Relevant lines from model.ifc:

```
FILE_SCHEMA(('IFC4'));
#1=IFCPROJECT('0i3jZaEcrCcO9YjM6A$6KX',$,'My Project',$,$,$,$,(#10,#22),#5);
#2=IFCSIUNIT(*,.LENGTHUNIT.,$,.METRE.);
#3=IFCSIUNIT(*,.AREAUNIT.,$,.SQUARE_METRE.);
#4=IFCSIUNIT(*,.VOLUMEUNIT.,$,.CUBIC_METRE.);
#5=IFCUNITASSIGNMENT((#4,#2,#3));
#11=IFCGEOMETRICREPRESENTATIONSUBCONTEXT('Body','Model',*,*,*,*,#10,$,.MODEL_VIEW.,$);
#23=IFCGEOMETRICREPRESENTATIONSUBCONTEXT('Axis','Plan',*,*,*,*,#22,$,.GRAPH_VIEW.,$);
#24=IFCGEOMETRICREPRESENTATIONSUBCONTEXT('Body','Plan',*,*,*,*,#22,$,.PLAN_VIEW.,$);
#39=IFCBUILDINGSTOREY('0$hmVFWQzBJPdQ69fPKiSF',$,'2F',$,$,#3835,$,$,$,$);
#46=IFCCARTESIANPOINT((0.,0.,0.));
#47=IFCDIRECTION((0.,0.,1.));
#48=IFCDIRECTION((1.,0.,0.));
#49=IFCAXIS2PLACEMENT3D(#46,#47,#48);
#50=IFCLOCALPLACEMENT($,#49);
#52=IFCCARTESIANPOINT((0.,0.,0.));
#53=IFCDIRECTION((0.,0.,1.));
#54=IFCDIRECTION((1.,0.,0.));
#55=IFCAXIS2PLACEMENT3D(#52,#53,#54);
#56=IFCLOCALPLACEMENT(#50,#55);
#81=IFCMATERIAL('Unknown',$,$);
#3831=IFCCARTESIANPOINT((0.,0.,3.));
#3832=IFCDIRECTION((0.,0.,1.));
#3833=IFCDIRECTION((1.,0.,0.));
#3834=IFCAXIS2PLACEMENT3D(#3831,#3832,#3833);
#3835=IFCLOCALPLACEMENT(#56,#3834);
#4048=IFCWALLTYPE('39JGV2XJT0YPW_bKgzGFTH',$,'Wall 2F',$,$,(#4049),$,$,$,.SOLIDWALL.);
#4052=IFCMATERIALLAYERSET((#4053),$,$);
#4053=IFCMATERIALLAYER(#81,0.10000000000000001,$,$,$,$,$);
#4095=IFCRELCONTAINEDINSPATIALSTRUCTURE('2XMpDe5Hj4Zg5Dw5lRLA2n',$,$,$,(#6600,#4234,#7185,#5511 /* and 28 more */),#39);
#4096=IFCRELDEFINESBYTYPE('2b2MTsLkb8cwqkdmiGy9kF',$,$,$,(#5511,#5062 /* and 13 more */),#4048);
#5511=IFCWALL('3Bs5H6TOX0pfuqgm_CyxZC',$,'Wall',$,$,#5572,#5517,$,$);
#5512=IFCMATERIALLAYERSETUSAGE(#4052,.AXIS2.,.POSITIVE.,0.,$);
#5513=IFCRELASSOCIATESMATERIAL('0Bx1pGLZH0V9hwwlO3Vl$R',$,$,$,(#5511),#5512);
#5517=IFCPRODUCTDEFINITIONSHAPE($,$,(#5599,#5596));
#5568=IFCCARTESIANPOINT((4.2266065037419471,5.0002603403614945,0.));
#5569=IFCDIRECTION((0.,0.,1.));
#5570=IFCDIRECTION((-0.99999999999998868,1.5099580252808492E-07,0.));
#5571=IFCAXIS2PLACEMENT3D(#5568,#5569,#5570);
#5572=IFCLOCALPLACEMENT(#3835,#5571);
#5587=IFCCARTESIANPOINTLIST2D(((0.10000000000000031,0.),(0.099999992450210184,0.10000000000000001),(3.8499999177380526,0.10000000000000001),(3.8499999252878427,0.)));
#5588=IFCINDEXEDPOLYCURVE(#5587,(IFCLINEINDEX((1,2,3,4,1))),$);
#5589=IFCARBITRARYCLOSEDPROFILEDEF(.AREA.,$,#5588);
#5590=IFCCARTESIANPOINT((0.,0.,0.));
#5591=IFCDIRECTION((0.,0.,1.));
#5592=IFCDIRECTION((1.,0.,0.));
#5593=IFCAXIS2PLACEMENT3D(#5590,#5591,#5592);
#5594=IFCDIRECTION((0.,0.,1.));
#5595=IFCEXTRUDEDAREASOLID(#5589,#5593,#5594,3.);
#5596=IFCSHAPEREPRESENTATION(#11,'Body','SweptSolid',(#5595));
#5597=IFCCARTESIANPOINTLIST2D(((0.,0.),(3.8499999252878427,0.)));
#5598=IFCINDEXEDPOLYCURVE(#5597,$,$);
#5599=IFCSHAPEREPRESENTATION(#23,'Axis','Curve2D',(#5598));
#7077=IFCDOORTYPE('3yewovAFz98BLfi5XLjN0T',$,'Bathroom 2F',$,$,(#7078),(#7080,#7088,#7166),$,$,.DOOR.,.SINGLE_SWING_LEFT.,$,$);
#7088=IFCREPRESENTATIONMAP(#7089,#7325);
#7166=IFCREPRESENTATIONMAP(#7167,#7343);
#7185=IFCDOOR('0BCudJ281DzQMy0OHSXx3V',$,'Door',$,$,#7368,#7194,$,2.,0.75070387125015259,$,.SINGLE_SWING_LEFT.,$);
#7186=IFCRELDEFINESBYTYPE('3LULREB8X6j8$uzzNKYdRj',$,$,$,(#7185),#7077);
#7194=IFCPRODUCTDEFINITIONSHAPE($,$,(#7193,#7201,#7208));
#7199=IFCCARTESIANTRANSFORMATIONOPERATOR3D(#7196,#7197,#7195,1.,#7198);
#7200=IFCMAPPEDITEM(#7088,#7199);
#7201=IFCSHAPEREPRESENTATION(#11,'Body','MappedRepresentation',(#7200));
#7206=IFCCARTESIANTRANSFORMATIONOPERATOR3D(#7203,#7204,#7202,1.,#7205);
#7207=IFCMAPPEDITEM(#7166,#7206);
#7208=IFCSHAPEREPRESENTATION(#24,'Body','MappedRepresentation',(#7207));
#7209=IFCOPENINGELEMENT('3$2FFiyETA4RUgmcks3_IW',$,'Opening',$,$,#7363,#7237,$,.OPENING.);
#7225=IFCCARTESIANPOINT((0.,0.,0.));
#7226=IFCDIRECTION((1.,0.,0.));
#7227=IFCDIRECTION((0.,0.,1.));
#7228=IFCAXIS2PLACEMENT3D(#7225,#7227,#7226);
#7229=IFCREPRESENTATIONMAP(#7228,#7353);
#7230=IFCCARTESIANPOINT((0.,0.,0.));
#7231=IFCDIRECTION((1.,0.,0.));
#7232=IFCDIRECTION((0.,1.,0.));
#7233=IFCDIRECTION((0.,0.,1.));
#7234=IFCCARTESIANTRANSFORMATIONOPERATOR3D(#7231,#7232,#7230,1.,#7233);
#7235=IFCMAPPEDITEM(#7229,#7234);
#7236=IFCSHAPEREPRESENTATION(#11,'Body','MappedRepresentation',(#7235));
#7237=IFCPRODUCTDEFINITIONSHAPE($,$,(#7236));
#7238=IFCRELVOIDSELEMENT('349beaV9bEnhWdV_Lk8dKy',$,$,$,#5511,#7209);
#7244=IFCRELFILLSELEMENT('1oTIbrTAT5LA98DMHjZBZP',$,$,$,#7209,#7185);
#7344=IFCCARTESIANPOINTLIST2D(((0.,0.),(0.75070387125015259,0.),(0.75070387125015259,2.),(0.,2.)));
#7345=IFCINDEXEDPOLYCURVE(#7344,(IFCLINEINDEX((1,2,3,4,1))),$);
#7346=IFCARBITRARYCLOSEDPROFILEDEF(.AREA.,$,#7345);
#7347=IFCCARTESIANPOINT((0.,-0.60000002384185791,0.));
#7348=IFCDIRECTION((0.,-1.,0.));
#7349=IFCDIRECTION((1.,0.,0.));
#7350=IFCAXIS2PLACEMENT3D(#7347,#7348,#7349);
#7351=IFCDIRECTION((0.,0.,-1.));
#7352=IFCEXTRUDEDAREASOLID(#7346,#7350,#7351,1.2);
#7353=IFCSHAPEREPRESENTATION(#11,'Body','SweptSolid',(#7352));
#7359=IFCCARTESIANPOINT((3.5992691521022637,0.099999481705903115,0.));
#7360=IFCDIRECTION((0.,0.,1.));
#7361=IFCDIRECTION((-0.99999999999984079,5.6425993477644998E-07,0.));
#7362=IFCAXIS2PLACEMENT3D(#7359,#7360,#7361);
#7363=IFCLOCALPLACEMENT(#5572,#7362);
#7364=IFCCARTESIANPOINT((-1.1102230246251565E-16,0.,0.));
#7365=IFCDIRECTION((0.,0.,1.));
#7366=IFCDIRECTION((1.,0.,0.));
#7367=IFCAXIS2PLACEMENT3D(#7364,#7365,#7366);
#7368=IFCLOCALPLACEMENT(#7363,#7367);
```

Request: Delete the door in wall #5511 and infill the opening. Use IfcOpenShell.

```python
import ifcopenshell
import ifcopenshell.api.feature
import ifcopenshell.api.root
import ifcopenshell.geom
import ifcopenshell.util.shape

model = ifcopenshell.open("model.ifc")
settings = ifcopenshell.geom.settings()


def volume(element):
    """Net volume in cubic metres, openings subtracted."""
    shape = ifcopenshell.geom.create_shape(settings, element)
    return ifcopenshell.util.shape.get_volume(shape.geometry)


door = model.by_id(7185)
opening = door.FillsVoids[0].RelatingOpeningElement
wall = opening.VoidsElements[0].RelatingBuildingElement
before = volume(wall)

ifcopenshell.api.root.remove_product(model, product=door)
ifcopenshell.api.feature.remove_feature(model, feature=opening)

after = volume(wall)

print(f"wall volume {before:.3f} -> {after:.3f} m3")

model.write("model_edited.ifc")
```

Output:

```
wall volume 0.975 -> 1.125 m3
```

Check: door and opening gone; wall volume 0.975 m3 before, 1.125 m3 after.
